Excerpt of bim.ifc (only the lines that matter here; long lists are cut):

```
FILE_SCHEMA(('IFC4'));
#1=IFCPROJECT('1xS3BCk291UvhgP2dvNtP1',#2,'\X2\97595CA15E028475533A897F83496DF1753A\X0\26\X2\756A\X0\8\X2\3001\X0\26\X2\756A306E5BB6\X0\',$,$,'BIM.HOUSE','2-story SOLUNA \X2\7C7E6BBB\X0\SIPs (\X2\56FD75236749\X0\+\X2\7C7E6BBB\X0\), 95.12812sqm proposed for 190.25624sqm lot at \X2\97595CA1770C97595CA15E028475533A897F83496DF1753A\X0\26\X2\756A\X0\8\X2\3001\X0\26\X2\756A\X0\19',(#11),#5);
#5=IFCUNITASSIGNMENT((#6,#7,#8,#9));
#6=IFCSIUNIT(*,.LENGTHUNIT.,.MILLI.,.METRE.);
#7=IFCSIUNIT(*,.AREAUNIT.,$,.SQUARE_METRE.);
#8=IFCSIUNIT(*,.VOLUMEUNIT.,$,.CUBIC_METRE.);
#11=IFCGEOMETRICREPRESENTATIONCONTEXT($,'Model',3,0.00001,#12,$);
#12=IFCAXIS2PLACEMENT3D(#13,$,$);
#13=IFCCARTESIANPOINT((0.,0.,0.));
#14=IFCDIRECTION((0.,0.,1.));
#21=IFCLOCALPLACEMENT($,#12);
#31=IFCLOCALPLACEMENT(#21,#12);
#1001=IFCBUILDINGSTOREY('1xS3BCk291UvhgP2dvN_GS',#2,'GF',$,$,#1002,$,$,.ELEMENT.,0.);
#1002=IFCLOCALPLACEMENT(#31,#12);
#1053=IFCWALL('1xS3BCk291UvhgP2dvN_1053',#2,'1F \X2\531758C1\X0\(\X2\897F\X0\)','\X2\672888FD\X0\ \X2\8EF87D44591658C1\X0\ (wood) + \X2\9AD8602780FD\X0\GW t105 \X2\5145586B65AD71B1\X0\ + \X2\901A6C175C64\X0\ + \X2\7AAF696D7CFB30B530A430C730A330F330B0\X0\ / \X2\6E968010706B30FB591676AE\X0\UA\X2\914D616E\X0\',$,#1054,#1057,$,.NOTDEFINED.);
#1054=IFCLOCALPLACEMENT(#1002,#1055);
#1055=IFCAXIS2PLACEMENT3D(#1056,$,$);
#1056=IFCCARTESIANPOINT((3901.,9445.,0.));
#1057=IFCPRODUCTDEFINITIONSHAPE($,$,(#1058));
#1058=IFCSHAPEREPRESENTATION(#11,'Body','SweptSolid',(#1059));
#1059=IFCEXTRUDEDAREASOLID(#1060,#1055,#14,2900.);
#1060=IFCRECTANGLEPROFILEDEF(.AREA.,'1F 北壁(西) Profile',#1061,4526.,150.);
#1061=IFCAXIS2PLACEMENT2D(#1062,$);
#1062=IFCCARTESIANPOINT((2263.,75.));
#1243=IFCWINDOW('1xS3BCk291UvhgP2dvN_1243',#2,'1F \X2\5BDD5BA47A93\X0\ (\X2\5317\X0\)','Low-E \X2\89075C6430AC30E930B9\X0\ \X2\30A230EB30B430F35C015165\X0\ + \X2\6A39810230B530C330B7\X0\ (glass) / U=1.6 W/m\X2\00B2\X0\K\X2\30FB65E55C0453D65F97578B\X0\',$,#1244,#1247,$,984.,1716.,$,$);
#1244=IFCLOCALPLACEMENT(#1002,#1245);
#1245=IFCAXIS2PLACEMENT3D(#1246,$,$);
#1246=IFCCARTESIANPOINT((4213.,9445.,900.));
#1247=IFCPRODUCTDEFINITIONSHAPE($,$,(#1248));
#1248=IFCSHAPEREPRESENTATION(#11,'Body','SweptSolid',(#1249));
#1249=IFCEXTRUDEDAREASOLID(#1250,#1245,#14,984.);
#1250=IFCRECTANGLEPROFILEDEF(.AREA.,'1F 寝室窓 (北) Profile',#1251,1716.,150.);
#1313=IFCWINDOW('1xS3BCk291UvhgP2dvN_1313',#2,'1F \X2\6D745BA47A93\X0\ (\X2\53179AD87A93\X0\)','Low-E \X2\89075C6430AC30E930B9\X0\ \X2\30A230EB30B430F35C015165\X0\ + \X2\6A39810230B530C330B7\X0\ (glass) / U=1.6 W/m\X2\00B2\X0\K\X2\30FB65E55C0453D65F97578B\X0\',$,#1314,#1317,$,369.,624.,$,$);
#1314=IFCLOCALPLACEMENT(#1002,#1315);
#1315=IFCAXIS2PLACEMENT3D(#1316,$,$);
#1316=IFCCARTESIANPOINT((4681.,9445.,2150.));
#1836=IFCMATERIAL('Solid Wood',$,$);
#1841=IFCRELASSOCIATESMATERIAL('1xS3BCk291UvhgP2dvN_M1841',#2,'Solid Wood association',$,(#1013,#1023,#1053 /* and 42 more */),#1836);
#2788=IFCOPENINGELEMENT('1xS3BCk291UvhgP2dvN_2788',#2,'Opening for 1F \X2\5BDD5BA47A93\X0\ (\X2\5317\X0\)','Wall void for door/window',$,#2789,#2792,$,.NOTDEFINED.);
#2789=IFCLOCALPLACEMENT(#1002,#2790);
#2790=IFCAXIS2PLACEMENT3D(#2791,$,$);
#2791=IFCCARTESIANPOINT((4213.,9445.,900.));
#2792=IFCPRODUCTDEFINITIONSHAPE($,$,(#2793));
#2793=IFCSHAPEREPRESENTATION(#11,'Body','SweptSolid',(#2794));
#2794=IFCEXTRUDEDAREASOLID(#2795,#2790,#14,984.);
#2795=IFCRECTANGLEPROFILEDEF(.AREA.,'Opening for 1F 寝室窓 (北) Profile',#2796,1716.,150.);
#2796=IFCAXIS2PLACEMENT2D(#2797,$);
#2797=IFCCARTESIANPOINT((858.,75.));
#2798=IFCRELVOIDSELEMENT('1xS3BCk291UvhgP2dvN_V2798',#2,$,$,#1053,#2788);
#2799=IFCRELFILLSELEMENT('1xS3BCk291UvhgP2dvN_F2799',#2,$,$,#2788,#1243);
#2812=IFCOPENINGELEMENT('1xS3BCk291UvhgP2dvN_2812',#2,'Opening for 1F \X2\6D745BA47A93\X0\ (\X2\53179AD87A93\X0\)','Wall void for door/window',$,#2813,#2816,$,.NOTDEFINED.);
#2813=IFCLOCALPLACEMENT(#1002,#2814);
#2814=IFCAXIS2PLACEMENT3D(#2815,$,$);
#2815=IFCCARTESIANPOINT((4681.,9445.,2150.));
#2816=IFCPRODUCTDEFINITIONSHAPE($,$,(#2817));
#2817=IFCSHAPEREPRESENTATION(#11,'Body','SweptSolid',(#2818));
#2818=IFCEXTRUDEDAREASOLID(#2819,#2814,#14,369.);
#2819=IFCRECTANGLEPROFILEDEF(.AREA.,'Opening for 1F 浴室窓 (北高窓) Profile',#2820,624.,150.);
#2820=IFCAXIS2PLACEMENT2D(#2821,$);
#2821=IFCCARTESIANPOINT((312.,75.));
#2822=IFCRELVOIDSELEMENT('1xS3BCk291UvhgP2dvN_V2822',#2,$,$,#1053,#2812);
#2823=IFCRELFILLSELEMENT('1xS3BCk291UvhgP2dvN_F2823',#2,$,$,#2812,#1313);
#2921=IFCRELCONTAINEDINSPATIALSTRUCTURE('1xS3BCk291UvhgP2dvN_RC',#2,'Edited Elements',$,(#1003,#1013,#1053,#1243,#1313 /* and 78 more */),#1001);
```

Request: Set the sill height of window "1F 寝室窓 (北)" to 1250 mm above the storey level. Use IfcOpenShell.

```python
import numpy as np
import ifcopenshell
import ifcopenshell.api.geometry
import ifcopenshell.geom
import ifcopenshell.util.element
import ifcopenshell.util.placement
import ifcopenshell.util.shape
import ifcopenshell.util.unit

model = ifcopenshell.open("bim.ifc")
unit_scale = ifcopenshell.util.unit.calculate_unit_scale(model)

window = model.by_id(1243)
opening = window.FillsVoids[0].RelatingOpeningElement
storey = ifcopenshell.util.element.get_container(window, ifc_class="IfcBuildingStorey")
level = ifcopenshell.util.placement.get_local_placement(storey.ObjectPlacement)[2, 3]

# The opening's origin need not be at the sill, so measure its lowest point.
shape = ifcopenshell.geom.create_shape(ifcopenshell.geom.settings(), opening)
bottom = ifcopenshell.util.shape.get_shape_bottom_elevation(shape, shape.geometry) / unit_scale
dz = level + 1.25 / unit_scale - bottom

shift = np.array([0.0, 0.0, dz])
# The window is not placed relative to its opening, so move both.
for product in (opening, window):
    matrix = ifcopenshell.util.placement.get_local_placement(product.ObjectPlacement)
    matrix[:3, 3] += shift
    ifcopenshell.api.geometry.edit_object_placement(model, product=product, matrix=matrix, is_si=False)

print(f"moved by {dz * unit_scale:+.3f} m")

model.write("bim_edited.ifc")
```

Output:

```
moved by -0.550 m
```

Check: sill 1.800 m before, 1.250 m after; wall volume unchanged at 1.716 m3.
